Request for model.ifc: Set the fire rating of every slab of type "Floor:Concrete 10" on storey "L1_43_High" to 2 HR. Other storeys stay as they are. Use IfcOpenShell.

First a look at what the model holds.

```python
import ifcopenshell
import ifcopenshell.util.element

model = ifcopenshell.open("model.ifc")
print(model.schema)
storey = next(s for s in model.by_type("IfcBuildingStorey") if s.Name == "L1_43_High")
slabs = [e for e in ifcopenshell.util.element.get_decomposition(storey) if e.is_a("IfcSlab")]
seen = {}
for e in slabs:
    element_type = ifcopenshell.util.element.get_type(e)
    key = (element_type.Name if element_type != e and element_type else None, ifcopenshell.util.element.get_pset(e, "Pset_SlabCommon", "FireRating"))
    seen[key] = seen.get(key, 0) + 1
for (name, value), count in sorted(seen.items(), key=str):
    print(count, "x", name, "|", value)
```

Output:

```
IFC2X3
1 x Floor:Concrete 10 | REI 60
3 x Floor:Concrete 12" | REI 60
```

```python
import ifcopenshell
import ifcopenshell.api.pset
import ifcopenshell.util.element

model = ifcopenshell.open("model.ifc")

storey = next(s for s in model.by_type("IfcBuildingStorey") if s.Name == "L1_43_High")
slabs = [e for e in ifcopenshell.util.element.get_decomposition(storey) if e.is_a("IfcSlab")]

count = 0
for e in slabs:
    element_type = ifcopenshell.util.element.get_type(e)
    if element_type in (None, e) or element_type.Name != "Floor:Concrete 10":
        continue
    # add_pset returns the element's existing set when there is one.
    pset = ifcopenshell.api.pset.add_pset(model, product=e, name="Pset_SlabCommon")
    ifcopenshell.api.pset.edit_pset(model, pset=pset, properties={"FireRating": "2 HR"})
    count += 1

print(count, "slabs updated")

model.write("model_rev.ifc")
```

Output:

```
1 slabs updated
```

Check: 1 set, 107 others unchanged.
